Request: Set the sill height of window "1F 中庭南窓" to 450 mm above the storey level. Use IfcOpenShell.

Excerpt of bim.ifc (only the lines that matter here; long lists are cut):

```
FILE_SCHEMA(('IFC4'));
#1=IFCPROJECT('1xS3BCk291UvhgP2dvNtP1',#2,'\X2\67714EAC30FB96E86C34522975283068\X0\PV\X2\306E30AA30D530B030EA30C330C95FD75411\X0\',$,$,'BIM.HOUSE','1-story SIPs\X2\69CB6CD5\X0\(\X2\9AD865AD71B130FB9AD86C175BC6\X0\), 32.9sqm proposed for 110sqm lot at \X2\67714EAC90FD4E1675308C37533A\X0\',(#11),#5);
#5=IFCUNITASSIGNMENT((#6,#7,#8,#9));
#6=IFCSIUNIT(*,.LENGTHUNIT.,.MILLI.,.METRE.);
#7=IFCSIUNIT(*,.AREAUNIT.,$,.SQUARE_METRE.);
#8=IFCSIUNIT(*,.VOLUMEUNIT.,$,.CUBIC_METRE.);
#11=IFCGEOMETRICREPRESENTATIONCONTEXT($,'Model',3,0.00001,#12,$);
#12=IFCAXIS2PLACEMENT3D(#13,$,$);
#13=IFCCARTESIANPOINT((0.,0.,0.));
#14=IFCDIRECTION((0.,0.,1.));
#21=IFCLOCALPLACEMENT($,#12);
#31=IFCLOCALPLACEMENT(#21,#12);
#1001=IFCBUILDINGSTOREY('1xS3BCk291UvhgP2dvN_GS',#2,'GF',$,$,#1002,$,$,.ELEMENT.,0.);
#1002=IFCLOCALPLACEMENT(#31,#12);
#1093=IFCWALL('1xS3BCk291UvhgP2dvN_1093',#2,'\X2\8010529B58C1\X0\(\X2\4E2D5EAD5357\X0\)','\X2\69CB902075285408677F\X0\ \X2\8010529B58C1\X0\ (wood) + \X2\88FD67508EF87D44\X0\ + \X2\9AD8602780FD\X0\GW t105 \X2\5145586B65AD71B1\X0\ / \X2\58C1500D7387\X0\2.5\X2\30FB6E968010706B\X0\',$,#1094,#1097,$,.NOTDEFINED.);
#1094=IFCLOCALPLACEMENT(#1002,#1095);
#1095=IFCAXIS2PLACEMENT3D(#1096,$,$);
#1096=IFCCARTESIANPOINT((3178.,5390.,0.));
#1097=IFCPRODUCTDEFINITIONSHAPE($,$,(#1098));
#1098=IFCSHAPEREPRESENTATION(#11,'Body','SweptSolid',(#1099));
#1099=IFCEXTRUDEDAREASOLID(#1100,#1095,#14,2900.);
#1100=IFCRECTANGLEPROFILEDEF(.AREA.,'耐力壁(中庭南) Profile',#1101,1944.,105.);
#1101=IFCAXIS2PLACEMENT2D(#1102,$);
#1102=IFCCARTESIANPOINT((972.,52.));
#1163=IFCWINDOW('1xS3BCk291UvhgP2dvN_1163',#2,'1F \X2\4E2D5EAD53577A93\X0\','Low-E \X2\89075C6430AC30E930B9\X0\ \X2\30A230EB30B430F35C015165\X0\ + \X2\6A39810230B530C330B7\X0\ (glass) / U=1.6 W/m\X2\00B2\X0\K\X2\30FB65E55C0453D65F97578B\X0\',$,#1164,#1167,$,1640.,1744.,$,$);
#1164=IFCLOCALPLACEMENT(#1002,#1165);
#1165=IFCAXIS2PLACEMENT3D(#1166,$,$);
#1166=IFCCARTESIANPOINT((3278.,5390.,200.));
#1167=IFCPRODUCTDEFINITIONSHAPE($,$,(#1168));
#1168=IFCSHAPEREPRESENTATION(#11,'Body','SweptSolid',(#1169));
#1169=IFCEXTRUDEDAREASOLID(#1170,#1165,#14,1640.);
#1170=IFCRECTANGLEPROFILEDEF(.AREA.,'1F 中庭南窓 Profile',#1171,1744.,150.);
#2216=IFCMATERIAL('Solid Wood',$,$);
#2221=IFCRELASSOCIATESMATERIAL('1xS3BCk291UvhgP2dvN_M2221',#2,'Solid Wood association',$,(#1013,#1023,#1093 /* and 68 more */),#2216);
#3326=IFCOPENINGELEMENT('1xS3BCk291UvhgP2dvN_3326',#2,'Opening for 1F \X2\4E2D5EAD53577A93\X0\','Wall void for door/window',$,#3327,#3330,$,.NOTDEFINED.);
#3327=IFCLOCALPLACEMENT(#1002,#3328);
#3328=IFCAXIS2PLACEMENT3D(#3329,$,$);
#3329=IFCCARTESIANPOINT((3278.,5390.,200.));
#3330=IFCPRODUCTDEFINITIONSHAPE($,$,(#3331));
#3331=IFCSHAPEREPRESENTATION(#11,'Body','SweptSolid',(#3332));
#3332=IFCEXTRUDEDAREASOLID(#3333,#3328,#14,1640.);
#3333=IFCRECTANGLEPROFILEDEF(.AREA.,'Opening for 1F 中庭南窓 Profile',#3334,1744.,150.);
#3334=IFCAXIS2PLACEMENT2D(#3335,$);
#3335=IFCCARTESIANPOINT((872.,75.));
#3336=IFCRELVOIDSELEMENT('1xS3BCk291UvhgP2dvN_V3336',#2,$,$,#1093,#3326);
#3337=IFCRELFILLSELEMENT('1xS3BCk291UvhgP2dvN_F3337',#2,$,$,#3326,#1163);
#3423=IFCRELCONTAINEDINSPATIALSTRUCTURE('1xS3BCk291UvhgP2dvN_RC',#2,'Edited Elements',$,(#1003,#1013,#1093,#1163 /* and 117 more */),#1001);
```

```python
import numpy as np
import ifcopenshell
import ifcopenshell.api.geometry
import ifcopenshell.geom
import ifcopenshell.util.element
import ifcopenshell.util.placement
import ifcopenshell.util.shape
import ifcopenshell.util.unit

model = ifcopenshell.open("bim.ifc")
unit_scale = ifcopenshell.util.unit.calculate_unit_scale(model)

window = model.by_id(1163)
opening = window.FillsVoids[0].RelatingOpeningElement
storey = ifcopenshell.util.element.get_container(window, ifc_class="IfcBuildingStorey")
level = ifcopenshell.util.placement.get_local_placement(storey.ObjectPlacement)[2, 3]

# The opening's origin need not be at the sill, so measure its lowest point.
shape = ifcopenshell.geom.create_shape(ifcopenshell.geom.settings(), opening)
bottom = ifcopenshell.util.shape.get_shape_bottom_elevation(shape, shape.geometry) / unit_scale
dz = level + 450.0 - bottom

shift = np.array([0.0, 0.0, dz])
# The window is not placed relative to its opening, so move both.
for product in (opening, window):
    matrix = ifcopenshell.util.placement.get_local_placement(product.ObjectPlacement)
    matrix[:3, 3] += shift
    ifcopenshell.api.geometry.edit_object_placement(model, product=product, matrix=matrix, is_si=False)

print(f"moved by {dz * unit_scale:+.3f} m")

model.write("bim_edited.ifc")
```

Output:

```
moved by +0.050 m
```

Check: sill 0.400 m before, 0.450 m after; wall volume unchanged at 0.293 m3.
